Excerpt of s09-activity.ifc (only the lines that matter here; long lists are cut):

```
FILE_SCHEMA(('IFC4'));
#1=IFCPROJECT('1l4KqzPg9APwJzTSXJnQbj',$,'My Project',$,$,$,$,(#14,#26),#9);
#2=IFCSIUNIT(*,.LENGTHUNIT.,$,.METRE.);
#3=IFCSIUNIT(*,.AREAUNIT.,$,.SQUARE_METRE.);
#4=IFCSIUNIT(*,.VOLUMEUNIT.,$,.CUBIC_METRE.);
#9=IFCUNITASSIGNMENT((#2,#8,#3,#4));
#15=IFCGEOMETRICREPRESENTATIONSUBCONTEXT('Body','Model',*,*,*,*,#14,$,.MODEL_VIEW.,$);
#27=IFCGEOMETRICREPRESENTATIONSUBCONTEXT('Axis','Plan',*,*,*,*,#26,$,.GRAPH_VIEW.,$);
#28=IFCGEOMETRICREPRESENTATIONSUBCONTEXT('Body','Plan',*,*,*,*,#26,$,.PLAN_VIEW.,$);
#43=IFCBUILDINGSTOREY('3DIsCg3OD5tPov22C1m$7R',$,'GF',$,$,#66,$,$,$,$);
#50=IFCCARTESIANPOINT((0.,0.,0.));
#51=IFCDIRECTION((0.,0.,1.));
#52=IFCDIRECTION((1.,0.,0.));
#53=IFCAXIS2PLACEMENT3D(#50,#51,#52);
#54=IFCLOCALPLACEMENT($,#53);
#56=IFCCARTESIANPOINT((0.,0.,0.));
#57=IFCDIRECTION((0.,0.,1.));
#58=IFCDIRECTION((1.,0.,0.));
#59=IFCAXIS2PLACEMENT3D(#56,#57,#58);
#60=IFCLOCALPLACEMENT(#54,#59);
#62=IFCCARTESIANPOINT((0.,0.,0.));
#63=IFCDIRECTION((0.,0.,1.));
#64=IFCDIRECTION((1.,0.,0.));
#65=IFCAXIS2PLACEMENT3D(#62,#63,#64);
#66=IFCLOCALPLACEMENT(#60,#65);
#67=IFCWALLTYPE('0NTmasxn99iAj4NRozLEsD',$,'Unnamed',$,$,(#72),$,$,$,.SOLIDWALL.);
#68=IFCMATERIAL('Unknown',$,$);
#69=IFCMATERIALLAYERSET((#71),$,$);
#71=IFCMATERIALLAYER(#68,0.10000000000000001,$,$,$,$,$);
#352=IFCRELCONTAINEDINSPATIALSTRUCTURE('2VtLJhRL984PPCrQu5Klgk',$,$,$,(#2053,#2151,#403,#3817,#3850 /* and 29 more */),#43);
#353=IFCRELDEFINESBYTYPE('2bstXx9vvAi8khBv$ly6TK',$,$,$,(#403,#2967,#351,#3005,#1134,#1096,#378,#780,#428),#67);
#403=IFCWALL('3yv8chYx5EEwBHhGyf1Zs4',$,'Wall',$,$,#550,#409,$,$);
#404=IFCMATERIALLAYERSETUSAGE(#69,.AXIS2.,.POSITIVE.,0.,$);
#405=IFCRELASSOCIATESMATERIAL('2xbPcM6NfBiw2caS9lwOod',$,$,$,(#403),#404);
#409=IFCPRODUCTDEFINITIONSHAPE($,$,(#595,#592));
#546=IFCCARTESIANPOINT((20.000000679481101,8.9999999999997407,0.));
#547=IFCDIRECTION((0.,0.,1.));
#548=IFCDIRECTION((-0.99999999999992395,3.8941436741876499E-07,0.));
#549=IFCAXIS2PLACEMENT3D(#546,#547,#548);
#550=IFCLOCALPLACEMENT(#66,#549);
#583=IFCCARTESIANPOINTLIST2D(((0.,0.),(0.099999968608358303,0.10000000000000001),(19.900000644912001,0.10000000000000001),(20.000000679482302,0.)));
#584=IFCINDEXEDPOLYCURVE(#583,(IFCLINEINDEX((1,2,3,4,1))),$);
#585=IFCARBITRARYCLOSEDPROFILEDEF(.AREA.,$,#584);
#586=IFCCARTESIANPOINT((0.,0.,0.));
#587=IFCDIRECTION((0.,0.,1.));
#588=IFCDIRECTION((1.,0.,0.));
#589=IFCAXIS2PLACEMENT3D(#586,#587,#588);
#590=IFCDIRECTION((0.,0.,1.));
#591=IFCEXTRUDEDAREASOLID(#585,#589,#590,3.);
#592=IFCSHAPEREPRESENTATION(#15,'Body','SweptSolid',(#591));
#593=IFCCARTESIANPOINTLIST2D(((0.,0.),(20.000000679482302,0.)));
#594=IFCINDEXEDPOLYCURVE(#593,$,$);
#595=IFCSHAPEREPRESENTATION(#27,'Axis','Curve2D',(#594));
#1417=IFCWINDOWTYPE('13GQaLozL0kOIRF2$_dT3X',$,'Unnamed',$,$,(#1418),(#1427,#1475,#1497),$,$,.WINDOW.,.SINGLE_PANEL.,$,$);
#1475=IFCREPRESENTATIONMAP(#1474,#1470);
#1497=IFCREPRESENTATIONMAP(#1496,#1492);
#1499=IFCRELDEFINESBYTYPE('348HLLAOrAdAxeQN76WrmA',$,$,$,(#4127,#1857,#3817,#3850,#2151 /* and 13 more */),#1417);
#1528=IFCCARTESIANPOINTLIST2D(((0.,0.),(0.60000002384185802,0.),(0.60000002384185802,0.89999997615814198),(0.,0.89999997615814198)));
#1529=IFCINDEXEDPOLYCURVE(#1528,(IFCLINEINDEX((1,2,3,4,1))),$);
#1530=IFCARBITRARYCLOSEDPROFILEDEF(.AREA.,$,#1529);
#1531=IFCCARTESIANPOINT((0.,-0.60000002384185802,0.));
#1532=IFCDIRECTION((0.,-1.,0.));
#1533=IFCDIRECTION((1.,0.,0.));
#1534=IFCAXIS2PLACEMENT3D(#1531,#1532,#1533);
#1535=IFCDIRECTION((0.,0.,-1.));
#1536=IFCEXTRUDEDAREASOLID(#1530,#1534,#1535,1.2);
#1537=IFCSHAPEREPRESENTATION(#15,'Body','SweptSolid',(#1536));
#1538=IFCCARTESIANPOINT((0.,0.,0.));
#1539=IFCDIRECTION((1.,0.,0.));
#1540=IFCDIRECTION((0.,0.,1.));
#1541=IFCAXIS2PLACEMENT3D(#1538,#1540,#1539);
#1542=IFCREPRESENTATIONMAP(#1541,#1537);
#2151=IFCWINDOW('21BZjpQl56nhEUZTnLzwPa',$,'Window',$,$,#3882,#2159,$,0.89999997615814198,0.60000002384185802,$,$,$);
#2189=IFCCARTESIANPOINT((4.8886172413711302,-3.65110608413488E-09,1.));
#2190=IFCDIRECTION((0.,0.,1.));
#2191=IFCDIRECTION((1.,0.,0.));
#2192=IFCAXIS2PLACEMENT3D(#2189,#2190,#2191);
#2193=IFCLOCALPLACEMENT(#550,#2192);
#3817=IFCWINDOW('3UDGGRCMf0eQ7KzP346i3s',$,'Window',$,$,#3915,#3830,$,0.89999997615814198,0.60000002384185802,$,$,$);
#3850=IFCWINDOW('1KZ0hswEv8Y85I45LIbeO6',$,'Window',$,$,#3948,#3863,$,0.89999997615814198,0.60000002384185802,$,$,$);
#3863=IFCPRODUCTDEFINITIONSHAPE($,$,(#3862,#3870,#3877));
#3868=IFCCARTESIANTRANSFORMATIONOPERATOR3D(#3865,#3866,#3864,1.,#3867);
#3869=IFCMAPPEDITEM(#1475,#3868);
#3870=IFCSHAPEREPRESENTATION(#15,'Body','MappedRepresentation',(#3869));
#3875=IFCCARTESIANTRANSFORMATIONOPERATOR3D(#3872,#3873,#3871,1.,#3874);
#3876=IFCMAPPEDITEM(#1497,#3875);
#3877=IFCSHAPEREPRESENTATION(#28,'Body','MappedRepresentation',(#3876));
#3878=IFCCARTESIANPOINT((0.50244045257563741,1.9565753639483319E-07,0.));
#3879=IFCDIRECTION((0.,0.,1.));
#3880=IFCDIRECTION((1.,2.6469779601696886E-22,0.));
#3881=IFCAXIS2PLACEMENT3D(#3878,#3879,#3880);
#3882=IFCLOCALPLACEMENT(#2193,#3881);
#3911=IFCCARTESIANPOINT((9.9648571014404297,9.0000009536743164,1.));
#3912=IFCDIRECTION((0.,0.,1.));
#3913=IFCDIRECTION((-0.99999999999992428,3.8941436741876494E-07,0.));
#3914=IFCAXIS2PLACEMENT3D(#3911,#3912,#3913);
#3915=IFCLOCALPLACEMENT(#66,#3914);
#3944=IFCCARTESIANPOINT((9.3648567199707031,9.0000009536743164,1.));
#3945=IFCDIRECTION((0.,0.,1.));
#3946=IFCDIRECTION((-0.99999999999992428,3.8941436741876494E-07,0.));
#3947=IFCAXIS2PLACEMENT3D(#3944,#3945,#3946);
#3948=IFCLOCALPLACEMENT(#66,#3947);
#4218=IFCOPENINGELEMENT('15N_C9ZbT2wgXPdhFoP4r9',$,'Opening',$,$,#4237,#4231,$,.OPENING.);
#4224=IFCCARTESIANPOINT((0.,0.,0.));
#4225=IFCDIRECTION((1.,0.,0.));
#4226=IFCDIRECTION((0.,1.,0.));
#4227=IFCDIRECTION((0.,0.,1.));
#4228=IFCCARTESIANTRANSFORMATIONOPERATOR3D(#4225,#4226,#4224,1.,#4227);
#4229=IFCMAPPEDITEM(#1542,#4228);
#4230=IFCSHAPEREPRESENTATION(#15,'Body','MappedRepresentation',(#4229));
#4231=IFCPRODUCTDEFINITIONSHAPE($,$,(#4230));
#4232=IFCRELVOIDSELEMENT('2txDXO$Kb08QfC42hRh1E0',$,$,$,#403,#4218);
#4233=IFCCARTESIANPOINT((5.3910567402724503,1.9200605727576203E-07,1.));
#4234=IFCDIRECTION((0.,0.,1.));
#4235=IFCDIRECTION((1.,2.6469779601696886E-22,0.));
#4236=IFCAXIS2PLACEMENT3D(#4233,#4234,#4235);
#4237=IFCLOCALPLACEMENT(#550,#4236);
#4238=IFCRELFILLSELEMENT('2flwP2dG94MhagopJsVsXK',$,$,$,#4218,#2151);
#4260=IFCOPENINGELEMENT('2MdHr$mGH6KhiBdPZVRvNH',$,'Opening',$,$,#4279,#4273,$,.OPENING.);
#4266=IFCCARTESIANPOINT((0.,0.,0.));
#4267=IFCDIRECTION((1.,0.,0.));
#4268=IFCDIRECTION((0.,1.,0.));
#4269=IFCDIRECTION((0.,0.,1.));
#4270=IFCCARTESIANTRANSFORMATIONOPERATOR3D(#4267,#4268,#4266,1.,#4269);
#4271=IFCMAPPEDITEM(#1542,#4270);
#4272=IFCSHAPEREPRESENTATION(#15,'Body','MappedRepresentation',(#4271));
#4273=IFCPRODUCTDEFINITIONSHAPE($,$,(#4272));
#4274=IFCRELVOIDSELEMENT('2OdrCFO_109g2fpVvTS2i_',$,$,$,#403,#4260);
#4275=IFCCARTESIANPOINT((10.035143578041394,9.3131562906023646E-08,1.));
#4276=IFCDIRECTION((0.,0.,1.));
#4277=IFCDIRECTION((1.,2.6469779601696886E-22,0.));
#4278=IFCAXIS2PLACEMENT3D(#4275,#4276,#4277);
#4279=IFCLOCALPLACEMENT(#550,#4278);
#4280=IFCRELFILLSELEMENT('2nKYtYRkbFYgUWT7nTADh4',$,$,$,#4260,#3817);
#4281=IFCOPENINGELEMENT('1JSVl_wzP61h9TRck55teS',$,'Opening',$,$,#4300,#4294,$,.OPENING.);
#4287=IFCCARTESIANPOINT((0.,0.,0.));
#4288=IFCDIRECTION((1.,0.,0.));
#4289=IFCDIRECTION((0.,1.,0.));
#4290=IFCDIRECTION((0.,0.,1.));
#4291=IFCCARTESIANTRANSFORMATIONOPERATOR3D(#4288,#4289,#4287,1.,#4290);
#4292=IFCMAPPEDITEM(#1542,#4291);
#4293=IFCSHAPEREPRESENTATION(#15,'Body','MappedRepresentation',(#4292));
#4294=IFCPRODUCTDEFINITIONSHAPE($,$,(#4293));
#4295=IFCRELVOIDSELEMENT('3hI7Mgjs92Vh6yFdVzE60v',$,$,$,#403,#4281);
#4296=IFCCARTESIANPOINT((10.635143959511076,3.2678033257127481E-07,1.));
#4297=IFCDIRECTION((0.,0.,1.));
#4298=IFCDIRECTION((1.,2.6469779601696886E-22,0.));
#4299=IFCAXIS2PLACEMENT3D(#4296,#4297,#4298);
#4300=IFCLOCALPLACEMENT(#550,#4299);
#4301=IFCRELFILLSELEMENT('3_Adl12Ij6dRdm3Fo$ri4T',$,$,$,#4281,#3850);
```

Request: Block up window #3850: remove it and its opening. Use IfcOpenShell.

```python
import ifcopenshell
import ifcopenshell.api.feature
import ifcopenshell.api.root
import ifcopenshell.geom
import ifcopenshell.util.shape

model = ifcopenshell.open("s09-activity.ifc")
settings = ifcopenshell.geom.settings()


def volume(element):
    """Net volume in cubic metres, openings subtracted."""
    shape = ifcopenshell.geom.create_shape(settings, element)
    return ifcopenshell.util.shape.get_volume(shape.geometry)


window = model.by_guid("1KZ0hswEv8Y85I45LIbeO6")
opening = window.FillsVoids[0].RelatingOpeningElement
wall = opening.VoidsElements[0].RelatingBuildingElement
before = volume(wall)

ifcopenshell.api.root.remove_product(model, product=window)
ifcopenshell.api.feature.remove_feature(model, feature=opening)

after = volume(wall)

print(f"wall volume {before:.3f} -> {after:.3f} m3")

model.write("s09-activity_updated.ifc")
```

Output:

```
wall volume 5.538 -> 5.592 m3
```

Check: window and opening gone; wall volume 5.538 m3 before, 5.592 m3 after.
